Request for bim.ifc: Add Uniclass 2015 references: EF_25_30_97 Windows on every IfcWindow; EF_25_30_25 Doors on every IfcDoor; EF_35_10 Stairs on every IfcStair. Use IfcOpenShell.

First a look at what the model holds.

```python
import ifcopenshell

model = ifcopenshell.open("bim.ifc")
print(model.schema)
print("classifications:", [c.Name for c in model.by_type("IfcClassification")])
for ifc_class in ("IfcDoor", "IfcRoof", "IfcStair", "IfcWall", "IfcWindow"):
    print(ifc_class, len(model.by_type(ifc_class)))
```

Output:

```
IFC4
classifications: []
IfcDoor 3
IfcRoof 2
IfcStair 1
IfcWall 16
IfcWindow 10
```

```python
import ifcopenshell
import ifcopenshell.api.classification

model = ifcopenshell.open("bim.ifc")

system = ifcopenshell.api.classification.add_classification(model, classification="Uniclass 2015")

codes = {
    "IfcWindow": ("EF_25_30_97", "Windows"),
    "IfcDoor": ("EF_25_30_25", "Doors"),
    "IfcStair": ("EF_35_10", "Stairs"),
}
for ifc_class, (code, name) in codes.items():
    products = model.by_type(ifc_class)
    ifcopenshell.api.classification.add_reference(
        model, products=products, classification=system, identification=code, name=name
    )
    print(code, len(products))

model.write("bim_updated.ifc")
```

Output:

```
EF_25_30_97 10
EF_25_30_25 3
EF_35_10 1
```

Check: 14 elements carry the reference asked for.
